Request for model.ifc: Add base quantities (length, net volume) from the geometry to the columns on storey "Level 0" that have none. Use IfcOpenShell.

First a look at what the model holds.

```python
import ifcopenshell
import ifcopenshell.util.element
import ifcopenshell.util.unit

model = ifcopenshell.open("model.ifc")
print(model.schema)
for unit_type in ("LENGTHUNIT", "AREAUNIT", "VOLUMEUNIT"):
    print(unit_type, ifcopenshell.util.unit.calculate_unit_scale(model, unit_type))
storey = next(s for s in model.by_type("IfcBuildingStorey") if s.Name == "Level 0")
columns = [e for e in ifcopenshell.util.element.get_decomposition(storey) if e.is_a("IfcColumn")]
for e in sorted(columns, key=lambda e: e.id()):
    print(e.id(), e.is_a(), e.Name, list(ifcopenshell.util.element.get_psets(e, qtos_only=True)), sep=" | ")
```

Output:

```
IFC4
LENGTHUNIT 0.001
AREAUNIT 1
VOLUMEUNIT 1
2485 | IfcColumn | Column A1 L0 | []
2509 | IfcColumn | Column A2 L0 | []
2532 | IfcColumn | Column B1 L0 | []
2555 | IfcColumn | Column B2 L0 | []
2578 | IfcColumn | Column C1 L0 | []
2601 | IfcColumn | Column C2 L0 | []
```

```python
import ifcopenshell
import ifcopenshell.api.pset
import ifcopenshell.geom
import ifcopenshell.util.element
import ifcopenshell.util.shape
import ifcopenshell.util.unit

model = ifcopenshell.open("model.ifc")
unit_scale = ifcopenshell.util.unit.calculate_unit_scale(model)
volume_scale = ifcopenshell.util.unit.calculate_unit_scale(model, "VOLUMEUNIT")
settings = ifcopenshell.geom.settings()

storey = next(s for s in model.by_type("IfcBuildingStorey") if s.Name == "Level 0")
columns = [e for e in ifcopenshell.util.element.get_decomposition(storey) if e.is_a("IfcColumn")]

for e in sorted(columns, key=lambda e: e.id()):
    if ifcopenshell.util.element.get_psets(e, qtos_only=True, should_inherit=False):
        continue
    # Geometry comes back in metres, in the element's own axes.
    shape = ifcopenshell.geom.create_shape(settings, e)
    values = {
        "Length": ifcopenshell.util.shape.get_z(shape.geometry) / unit_scale,
        "NetVolume": ifcopenshell.util.shape.get_volume(shape.geometry) / volume_scale,
    }
    qto = ifcopenshell.api.pset.add_qto(model, product=e, name="Qto_ColumnBaseQuantities")
    ifcopenshell.api.pset.edit_qto(model, qto=qto, properties=values)
    print(e.id(), {k: round(v, 3) for k, v in values.items()})

model.write("model_updated.ifc")
```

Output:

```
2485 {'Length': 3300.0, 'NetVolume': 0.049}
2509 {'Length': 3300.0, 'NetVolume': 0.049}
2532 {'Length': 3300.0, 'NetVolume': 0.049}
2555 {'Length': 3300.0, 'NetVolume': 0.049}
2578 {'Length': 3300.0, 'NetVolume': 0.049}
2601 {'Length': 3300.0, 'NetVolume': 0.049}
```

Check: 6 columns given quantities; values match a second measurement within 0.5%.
